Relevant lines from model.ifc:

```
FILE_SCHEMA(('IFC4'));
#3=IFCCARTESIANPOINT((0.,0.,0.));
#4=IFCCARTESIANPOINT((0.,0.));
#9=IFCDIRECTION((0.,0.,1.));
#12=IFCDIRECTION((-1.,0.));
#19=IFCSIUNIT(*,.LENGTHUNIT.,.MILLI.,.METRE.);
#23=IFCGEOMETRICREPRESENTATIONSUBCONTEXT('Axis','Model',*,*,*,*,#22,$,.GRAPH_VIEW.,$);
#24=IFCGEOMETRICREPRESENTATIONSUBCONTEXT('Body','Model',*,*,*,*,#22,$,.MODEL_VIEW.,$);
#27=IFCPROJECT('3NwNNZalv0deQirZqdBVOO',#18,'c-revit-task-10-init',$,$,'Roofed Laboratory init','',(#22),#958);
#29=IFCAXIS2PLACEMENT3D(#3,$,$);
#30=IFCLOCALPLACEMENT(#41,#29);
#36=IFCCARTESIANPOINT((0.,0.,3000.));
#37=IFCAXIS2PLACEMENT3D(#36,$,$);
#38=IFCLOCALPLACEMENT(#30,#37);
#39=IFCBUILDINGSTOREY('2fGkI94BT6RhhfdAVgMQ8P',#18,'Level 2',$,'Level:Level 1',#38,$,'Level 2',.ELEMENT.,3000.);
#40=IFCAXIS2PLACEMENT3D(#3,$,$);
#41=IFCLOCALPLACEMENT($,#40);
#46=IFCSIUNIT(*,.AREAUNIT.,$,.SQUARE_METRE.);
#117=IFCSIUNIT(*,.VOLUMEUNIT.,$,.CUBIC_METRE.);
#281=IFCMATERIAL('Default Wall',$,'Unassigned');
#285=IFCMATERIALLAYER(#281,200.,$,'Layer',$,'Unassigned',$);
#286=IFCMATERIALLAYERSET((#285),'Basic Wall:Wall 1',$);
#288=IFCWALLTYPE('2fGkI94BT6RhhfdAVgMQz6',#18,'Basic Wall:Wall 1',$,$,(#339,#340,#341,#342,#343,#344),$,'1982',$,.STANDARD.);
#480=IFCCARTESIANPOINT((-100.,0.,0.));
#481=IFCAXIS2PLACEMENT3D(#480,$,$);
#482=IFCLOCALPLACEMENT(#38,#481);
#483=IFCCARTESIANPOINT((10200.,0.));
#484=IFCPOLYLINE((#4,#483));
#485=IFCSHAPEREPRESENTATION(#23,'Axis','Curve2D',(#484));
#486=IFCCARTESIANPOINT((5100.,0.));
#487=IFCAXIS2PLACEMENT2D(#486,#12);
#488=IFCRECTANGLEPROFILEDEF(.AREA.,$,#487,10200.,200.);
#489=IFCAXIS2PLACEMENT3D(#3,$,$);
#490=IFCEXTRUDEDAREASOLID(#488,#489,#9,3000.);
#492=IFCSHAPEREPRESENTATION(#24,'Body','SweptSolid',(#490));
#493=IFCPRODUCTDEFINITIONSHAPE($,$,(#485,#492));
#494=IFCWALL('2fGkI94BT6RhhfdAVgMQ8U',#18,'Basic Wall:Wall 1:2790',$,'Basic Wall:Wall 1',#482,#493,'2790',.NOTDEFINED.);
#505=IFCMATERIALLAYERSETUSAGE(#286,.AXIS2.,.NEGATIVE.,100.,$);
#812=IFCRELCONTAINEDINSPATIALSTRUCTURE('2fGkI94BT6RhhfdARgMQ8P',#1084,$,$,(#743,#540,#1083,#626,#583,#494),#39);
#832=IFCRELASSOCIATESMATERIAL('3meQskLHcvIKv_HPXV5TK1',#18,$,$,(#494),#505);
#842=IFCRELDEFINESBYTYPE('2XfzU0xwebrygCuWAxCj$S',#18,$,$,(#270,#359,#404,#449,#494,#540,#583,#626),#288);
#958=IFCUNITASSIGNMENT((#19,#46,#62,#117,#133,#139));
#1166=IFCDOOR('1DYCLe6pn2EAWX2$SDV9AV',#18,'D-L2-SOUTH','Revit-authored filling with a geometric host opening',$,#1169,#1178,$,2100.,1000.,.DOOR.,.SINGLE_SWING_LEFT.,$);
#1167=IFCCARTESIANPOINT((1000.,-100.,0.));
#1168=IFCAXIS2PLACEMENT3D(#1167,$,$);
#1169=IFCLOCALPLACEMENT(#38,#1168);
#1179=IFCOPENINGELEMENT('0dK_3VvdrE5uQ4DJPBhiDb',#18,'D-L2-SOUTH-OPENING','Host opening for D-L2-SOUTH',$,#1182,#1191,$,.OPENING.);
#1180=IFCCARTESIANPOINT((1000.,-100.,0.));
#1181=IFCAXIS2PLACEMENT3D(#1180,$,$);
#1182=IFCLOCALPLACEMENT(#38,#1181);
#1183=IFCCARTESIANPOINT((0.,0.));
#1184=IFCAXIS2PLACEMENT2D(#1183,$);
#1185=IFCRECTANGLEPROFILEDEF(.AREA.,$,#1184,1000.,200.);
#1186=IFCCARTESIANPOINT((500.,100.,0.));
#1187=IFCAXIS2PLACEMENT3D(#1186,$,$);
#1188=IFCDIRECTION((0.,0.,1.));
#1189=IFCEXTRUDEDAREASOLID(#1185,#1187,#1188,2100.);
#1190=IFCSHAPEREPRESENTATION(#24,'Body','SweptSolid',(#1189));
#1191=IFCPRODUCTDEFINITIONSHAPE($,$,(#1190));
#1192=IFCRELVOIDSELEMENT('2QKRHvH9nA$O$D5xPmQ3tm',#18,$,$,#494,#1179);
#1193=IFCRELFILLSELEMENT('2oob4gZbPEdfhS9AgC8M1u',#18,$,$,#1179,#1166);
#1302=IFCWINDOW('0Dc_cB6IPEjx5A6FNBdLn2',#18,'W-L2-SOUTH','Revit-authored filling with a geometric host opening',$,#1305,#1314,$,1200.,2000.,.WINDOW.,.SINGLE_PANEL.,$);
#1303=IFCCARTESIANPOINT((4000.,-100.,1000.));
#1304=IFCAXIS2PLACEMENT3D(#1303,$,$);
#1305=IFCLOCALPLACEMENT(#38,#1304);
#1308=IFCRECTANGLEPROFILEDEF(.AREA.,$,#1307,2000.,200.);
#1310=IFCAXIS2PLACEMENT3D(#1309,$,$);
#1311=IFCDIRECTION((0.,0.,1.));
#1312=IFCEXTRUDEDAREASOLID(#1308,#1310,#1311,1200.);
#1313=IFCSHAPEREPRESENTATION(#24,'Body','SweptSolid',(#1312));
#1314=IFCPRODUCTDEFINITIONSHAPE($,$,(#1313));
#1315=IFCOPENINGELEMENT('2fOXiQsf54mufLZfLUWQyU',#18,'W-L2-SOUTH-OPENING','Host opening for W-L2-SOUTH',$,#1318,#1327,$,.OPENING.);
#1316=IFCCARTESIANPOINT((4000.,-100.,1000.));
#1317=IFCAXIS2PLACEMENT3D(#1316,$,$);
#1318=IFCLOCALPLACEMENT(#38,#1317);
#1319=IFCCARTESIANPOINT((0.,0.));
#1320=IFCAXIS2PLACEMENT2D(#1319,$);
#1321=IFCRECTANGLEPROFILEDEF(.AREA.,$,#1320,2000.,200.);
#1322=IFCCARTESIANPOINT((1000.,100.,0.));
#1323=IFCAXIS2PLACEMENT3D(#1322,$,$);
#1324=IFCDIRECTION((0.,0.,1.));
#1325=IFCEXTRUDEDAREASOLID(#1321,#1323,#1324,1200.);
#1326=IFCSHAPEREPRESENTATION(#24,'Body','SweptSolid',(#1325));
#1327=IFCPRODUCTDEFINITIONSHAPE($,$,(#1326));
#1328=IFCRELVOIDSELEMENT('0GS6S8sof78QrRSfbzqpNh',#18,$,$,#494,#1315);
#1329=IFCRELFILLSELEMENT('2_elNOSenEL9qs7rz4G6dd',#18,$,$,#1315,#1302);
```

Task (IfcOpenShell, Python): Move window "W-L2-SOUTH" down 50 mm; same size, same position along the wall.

```python
import numpy as np
import ifcopenshell
import ifcopenshell.api.geometry
import ifcopenshell.util.placement
import ifcopenshell.util.unit

model = ifcopenshell.open("model.ifc")
unit_scale = ifcopenshell.util.unit.calculate_unit_scale(model)

window = model.by_guid("0Dc_cB6IPEjx5A6FNBdLn2")
opening = window.FillsVoids[0].RelatingOpeningElement
dz = -0.05 / unit_scale

shift = np.array([0.0, 0.0, dz])
# The window is not placed relative to its opening, so move both.
for product in (opening, window):
    matrix = ifcopenshell.util.placement.get_local_placement(product.ObjectPlacement)
    matrix[:3, 3] += shift
    ifcopenshell.api.geometry.edit_object_placement(model, product=product, matrix=matrix, is_si=False)

print(f"moved by {dz * unit_scale:+.3f} m")

model.write("model-out.ifc")
```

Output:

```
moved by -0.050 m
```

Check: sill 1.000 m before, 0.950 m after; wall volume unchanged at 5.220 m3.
